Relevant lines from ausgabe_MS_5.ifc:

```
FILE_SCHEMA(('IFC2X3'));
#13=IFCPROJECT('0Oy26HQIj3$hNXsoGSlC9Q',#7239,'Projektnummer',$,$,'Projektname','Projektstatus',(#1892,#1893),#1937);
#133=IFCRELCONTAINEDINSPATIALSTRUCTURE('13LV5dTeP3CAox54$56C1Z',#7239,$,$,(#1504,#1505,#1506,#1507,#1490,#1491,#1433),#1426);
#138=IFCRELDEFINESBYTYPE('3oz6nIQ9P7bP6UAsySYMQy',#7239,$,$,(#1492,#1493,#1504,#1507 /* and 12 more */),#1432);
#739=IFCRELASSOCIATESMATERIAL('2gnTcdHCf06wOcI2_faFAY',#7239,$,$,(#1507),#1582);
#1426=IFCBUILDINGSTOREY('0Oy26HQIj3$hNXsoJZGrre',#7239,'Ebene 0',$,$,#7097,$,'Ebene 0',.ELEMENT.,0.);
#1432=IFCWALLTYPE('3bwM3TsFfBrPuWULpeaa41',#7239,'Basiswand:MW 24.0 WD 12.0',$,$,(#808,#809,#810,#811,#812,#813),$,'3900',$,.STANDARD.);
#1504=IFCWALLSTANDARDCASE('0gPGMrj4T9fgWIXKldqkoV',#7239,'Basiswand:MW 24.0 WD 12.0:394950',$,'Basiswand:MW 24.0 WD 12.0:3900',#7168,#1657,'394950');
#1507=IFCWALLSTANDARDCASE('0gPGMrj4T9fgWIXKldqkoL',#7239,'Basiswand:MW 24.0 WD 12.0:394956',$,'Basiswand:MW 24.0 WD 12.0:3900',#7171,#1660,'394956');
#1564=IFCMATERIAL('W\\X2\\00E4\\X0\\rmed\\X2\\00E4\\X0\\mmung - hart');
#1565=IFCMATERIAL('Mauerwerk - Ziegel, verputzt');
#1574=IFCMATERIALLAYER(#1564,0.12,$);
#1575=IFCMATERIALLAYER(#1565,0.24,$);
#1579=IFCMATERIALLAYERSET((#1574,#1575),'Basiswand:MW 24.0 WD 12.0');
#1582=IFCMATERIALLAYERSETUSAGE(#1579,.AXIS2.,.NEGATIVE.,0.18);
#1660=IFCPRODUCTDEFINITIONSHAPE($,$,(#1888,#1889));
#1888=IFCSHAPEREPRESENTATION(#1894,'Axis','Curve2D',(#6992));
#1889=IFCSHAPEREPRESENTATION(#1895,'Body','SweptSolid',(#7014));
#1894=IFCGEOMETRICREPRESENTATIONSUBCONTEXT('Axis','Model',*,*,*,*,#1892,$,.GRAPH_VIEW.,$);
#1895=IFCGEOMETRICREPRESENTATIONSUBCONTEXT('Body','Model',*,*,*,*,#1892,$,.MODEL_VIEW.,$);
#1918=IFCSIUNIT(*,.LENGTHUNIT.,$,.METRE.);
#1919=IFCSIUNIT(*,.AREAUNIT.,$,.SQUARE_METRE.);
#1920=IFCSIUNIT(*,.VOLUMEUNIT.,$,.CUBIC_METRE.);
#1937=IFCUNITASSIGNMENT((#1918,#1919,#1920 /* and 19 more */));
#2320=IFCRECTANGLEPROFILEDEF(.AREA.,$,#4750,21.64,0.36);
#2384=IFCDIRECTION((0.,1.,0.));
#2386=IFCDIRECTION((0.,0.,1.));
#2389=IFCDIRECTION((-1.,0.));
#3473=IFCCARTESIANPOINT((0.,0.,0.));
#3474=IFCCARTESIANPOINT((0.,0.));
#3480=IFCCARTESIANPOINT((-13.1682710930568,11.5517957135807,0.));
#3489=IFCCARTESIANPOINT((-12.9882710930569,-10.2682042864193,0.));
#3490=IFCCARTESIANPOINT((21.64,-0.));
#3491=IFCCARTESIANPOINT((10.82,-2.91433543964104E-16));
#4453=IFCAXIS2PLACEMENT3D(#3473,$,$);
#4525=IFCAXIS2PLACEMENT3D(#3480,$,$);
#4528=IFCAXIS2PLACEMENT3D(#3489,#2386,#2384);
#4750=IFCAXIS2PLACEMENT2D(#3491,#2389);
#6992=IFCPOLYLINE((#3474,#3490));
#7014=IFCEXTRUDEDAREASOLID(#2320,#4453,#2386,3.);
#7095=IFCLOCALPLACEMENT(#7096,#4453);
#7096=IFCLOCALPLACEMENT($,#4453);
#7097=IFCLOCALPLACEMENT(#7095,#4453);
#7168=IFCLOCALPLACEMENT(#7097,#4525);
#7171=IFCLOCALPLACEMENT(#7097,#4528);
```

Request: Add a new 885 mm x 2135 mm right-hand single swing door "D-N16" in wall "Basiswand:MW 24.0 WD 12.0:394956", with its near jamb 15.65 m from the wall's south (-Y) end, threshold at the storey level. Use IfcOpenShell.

```python
import numpy as np
import ifcopenshell
import ifcopenshell.api.feature
import ifcopenshell.api.geometry
import ifcopenshell.api.root
import ifcopenshell.api.spatial
import ifcopenshell.api.type
import ifcopenshell.geom
import ifcopenshell.util.element
import ifcopenshell.util.placement
import ifcopenshell.util.representation
import ifcopenshell.util.shape
import ifcopenshell.util.unit

model = ifcopenshell.open("ausgabe_MS_5.ifc")
unit_scale = ifcopenshell.util.unit.calculate_unit_scale(model)
settings = ifcopenshell.geom.settings()


def volume(element):
    """Net volume in cubic metres, openings subtracted."""
    shape = ifcopenshell.geom.create_shape(settings, element)
    return ifcopenshell.util.shape.get_volume(shape.geometry)


wall = model.by_guid("0gPGMrj4T9fgWIXKldqkoL")
storey = ifcopenshell.util.element.get_container(wall, ifc_class="IfcBuildingStorey")
context = ifcopenshell.util.representation.get_context(model, "Model", "Body", "MODEL_VIEW")
before = volume(wall)

width, height, from_end, sill = 0.885, 2.135, 15.65, 0.0  # metres

# The wall runs along its own X axis, and the end named is its -X end.
wall_shape = ifcopenshell.geom.create_shape(settings, wall)
x, y, z = ifcopenshell.util.shape.get_vertices(wall_shape.geometry).T
start = x.min() + from_end
face, thickness = float(y.min()), float(y.max() - y.min())
wall_matrix = ifcopenshell.util.placement.get_local_placement(wall.ObjectPlacement)
level = ifcopenshell.util.placement.get_local_placement(storey.ObjectPlacement)[2, 3]


def in_wall(x, y):
    """Placement at x, y metres in the wall's axes, at sill height."""
    matrix = wall_matrix.copy()
    matrix[:, 3] = wall_matrix @ np.array([x / unit_scale, y / unit_scale, 0.0, 1.0])
    matrix[2, 3] = level + sill / unit_scale
    return matrix


# Opening: a box that overshoots both wall faces by 50 mm.
opening = ifcopenshell.api.root.create_entity(model, ifc_class="IfcOpeningElement")
box = ifcopenshell.api.geometry.add_wall_representation(
    model, context=context, length=width, height=height, thickness=thickness + 0.1
)
ifcopenshell.api.geometry.assign_representation(model, product=opening, representation=box)
ifcopenshell.api.geometry.edit_object_placement(model, product=opening, matrix=in_wall(start, face - 0.05), is_si=False)
ifcopenshell.api.feature.add_feature(model, feature=opening, element=wall)

door = ifcopenshell.api.root.create_entity(model, ifc_class="IfcDoor", name="D-N16")
door.OverallWidth, door.OverallHeight = width / unit_scale, height / unit_scale
body = ifcopenshell.api.geometry.add_door_representation(
    model,
    context=context,
    overall_width=door.OverallWidth,
    overall_height=door.OverallHeight,
    operation_type="SINGLE_SWING_RIGHT",
    lining_properties={"LiningDepth": thickness / unit_scale, "ThresholdDepth": thickness / unit_scale},
)
ifcopenshell.api.geometry.assign_representation(model, product=door, representation=body)
ifcopenshell.api.spatial.assign_container(model, products=[door], relating_structure=storey)
fills = ifcopenshell.api.feature.add_filling(model, opening=opening, element=door)
fills.OwnerHistory = door.OwnerHistory  # required in IFC2X3

# IFC2X3 keeps the operation on the door style.
style = ifcopenshell.api.root.create_entity(model, ifc_class="IfcDoorStyle", name="D-N16")
style.OperationType, style.ConstructionType = "SINGLE_SWING_RIGHT", "NOTDEFINED"
style.ParameterTakesPrecedence = style.Sizeable = False
ifcopenshell.api.type.assign_type(model, related_objects=[door], relating_type=style)

# The lining spans the wall, so the door starts at the wall face.
ifcopenshell.api.geometry.edit_object_placement(model, product=door, matrix=in_wall(start, face), is_si=False)

after = volume(wall)

print(f"wall volume {before:.3f} -> {after:.3f} m3")

model.write("ausgabe_MS_5_v2.ifc")
```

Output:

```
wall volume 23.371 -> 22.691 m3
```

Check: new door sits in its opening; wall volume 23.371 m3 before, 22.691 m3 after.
